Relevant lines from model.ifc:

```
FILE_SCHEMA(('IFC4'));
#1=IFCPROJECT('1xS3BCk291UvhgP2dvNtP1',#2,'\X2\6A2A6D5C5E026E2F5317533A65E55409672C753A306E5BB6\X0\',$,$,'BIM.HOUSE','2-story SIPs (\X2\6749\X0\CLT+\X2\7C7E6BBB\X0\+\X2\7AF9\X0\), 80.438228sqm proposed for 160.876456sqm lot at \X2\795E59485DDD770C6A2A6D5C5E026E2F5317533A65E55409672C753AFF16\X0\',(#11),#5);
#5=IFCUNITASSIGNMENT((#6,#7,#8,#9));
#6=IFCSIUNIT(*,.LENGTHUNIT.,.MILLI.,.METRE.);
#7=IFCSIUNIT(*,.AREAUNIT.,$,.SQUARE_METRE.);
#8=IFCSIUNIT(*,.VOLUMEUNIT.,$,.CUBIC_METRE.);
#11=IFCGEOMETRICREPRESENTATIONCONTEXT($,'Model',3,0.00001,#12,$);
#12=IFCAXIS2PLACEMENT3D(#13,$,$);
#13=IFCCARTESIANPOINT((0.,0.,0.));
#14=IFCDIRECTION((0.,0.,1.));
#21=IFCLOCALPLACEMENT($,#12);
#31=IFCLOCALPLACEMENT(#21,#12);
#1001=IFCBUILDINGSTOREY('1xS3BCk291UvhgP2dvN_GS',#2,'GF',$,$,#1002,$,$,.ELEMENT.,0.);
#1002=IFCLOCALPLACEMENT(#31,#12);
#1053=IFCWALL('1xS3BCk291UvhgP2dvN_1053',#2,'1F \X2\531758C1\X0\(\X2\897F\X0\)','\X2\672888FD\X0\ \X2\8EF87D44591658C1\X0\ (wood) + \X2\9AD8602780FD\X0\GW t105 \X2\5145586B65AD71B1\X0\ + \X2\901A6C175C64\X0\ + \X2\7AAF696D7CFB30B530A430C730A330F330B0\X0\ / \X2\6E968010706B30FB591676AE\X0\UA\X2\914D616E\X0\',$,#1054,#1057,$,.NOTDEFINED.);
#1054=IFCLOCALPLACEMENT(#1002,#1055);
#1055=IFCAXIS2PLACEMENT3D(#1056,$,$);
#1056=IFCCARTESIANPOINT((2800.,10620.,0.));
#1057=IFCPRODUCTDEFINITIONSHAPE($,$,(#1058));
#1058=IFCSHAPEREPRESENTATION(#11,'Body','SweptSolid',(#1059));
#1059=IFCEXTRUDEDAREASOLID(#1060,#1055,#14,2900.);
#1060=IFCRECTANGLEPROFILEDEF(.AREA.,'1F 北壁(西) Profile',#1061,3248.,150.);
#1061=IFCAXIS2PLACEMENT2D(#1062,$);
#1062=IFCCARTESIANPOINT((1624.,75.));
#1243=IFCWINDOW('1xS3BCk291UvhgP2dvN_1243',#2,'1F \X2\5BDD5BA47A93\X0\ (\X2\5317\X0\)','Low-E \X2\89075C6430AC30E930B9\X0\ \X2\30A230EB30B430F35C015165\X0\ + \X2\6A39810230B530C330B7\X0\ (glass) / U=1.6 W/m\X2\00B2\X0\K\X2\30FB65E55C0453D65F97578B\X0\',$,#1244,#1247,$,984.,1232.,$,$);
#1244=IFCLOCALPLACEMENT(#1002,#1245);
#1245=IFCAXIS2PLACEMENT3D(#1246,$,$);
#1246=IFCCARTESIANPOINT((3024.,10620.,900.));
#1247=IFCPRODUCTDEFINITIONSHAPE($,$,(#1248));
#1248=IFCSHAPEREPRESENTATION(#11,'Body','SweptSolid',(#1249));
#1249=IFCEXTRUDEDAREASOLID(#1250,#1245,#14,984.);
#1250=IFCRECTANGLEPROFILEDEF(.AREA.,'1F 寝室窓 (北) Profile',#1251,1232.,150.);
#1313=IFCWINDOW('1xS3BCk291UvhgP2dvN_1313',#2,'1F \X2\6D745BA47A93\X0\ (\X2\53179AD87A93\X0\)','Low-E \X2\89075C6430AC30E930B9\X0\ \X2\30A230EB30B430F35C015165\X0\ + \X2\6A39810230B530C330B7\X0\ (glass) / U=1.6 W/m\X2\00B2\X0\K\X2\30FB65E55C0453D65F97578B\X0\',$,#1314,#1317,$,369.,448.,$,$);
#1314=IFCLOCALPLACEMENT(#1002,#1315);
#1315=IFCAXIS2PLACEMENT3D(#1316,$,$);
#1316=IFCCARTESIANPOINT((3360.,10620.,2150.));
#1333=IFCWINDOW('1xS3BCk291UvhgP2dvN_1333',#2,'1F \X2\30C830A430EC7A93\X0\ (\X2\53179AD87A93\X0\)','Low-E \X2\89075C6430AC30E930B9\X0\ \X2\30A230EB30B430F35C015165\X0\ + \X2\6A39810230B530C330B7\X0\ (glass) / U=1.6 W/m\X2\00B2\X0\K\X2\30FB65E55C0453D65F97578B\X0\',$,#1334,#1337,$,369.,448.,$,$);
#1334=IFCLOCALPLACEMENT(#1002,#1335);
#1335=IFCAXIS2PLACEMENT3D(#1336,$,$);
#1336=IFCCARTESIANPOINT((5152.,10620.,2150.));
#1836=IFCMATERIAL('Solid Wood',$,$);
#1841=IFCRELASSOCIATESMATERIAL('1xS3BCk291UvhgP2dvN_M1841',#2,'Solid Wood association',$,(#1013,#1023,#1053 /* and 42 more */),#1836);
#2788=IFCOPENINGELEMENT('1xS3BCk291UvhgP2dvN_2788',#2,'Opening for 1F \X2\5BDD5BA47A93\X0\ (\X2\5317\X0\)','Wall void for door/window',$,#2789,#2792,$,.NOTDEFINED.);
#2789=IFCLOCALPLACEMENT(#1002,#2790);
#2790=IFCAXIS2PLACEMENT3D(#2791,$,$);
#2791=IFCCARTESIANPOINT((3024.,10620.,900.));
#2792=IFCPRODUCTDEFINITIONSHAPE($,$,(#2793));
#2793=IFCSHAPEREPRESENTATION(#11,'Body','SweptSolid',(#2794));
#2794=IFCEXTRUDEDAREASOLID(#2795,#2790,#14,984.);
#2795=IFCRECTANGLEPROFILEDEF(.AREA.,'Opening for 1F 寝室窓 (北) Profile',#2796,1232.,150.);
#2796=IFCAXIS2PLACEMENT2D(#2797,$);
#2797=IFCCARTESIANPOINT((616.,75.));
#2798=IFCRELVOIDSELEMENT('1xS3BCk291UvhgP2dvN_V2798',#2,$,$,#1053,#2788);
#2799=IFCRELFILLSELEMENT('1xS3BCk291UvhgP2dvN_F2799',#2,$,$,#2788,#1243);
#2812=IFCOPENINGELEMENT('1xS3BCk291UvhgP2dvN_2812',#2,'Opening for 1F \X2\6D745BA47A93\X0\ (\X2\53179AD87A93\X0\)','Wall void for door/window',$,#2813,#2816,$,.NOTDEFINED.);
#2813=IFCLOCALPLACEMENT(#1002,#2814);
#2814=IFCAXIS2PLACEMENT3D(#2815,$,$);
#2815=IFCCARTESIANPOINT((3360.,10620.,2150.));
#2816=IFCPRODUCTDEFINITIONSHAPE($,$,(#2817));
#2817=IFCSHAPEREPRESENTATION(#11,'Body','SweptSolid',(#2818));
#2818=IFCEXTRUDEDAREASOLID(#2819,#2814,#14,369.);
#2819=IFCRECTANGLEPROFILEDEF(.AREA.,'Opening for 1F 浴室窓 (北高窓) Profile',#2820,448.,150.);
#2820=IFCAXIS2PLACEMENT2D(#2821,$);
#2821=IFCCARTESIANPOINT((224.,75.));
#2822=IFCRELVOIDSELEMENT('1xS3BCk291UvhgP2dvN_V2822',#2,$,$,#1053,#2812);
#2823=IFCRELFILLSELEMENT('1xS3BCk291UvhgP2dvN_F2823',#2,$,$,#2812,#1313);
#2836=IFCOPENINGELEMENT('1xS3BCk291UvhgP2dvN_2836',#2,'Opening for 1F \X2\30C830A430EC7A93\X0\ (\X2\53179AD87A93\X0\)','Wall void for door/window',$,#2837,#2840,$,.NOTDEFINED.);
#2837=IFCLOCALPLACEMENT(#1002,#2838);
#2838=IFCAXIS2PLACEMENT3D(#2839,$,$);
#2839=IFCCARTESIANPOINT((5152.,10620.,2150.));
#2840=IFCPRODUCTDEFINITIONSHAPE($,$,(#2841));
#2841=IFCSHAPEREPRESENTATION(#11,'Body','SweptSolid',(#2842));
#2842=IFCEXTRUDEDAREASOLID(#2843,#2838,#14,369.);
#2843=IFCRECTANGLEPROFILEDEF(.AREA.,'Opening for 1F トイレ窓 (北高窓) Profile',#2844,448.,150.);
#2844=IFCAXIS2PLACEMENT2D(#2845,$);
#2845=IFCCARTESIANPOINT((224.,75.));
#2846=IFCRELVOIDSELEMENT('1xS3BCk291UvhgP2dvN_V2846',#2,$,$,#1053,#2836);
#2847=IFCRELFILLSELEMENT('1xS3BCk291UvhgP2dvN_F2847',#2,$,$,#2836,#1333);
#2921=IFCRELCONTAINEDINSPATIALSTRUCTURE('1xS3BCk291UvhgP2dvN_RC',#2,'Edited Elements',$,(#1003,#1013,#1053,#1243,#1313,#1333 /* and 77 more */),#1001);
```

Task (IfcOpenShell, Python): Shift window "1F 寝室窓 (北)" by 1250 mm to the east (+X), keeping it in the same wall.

```python
import ifcopenshell
import ifcopenshell.api.geometry
import ifcopenshell.util.placement

model = ifcopenshell.open("model.ifc")

window = model.by_id(1243)
opening = window.FillsVoids[0].RelatingOpeningElement
wall = opening.VoidsElements[0].RelatingBuildingElement

wall_matrix = ifcopenshell.util.placement.get_local_placement(wall.ObjectPlacement)
shift = wall_matrix[:3, 0] * 1250.0
before = ifcopenshell.util.placement.get_local_placement(window.ObjectPlacement)[:3, 3].copy()

# The window is not placed relative to its opening, so move both.
for product in (opening, window):
    matrix = ifcopenshell.util.placement.get_local_placement(product.ObjectPlacement)
    matrix[:3, 3] += shift
    ifcopenshell.api.geometry.edit_object_placement(model, product=product, matrix=matrix, is_si=False)

after = ifcopenshell.util.placement.get_local_placement(window.ObjectPlacement)[:3, 3]
print("window moved by", (after - before).round(3) + 0.0)

model.write("model_edited.ifc")
```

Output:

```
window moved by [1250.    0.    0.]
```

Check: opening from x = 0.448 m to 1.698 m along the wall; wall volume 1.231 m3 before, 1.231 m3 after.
